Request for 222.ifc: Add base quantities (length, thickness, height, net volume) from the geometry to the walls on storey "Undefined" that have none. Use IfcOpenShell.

First a look at what the model holds.

```python
import ifcopenshell
import ifcopenshell.util.element
import ifcopenshell.util.unit

model = ifcopenshell.open("222.ifc")
print(model.schema)
for unit_type in ("LENGTHUNIT", "AREAUNIT", "VOLUMEUNIT"):
    print(unit_type, ifcopenshell.util.unit.calculate_unit_scale(model, unit_type))
storey = next(s for s in model.by_type("IfcBuildingStorey") if s.Name == "Undefined")
walls = [e for e in ifcopenshell.util.element.get_decomposition(storey) if e.is_a("IfcWall")]
for e in sorted(walls, key=lambda e: e.id()):
    print(e.id(), e.is_a(), e.Name, list(ifcopenshell.util.element.get_psets(e, qtos_only=True)), sep=" | ")
```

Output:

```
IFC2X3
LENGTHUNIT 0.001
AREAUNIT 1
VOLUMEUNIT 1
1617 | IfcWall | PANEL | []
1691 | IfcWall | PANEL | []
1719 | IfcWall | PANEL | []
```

```python
import ifcopenshell
import ifcopenshell.api.pset
import ifcopenshell.geom
import ifcopenshell.util.element
import ifcopenshell.util.shape
import ifcopenshell.util.unit

model = ifcopenshell.open("222.ifc")
unit_scale = ifcopenshell.util.unit.calculate_unit_scale(model)
volume_scale = ifcopenshell.util.unit.calculate_unit_scale(model, "VOLUMEUNIT")
settings = ifcopenshell.geom.settings()

storey = next(s for s in model.by_type("IfcBuildingStorey") if s.Name == "Undefined")
walls = [e for e in ifcopenshell.util.element.get_decomposition(storey) if e.is_a("IfcWall")]

for e in sorted(walls, key=lambda e: e.id()):
    if ifcopenshell.util.element.get_psets(e, qtos_only=True, should_inherit=False):
        continue
    # Geometry comes back in metres, in the element's own axes.
    shape = ifcopenshell.geom.create_shape(settings, e)
    values = {
        "Length": ifcopenshell.util.shape.get_x(shape.geometry) / unit_scale,
        "Width": ifcopenshell.util.shape.get_y(shape.geometry) / unit_scale,
        "Height": ifcopenshell.util.shape.get_z(shape.geometry) / unit_scale,
        "NetVolume": ifcopenshell.util.shape.get_volume(shape.geometry) / volume_scale,
    }
    qto = ifcopenshell.api.pset.add_qto(model, product=e, name="BaseQuantities")
    ifcopenshell.api.pset.edit_qto(model, qto=qto, properties=values)
    print(e.id(), {k: round(v, 3) for k, v in values.items()})

model.write("222_rev.ifc")
```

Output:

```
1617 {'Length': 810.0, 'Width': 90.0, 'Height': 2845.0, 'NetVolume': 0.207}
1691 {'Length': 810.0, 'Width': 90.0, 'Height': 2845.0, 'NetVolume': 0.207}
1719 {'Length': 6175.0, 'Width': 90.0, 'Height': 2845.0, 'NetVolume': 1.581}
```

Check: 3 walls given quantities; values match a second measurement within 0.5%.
